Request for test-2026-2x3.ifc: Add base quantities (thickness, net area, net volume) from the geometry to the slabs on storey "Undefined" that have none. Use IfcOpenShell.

First a look at what the model holds.

```python
import ifcopenshell
import ifcopenshell.util.element
import ifcopenshell.util.unit

model = ifcopenshell.open("test-2026-2x3.ifc")
print(model.schema)
for unit_type in ("LENGTHUNIT", "AREAUNIT", "VOLUMEUNIT"):
    print(unit_type, ifcopenshell.util.unit.calculate_unit_scale(model, unit_type))
storey = next(s for s in model.by_type("IfcBuildingStorey") if s.Name == "Undefined")
slabs = [e for e in ifcopenshell.util.element.get_decomposition(storey) if e.is_a("IfcSlab")]
for e in sorted(slabs, key=lambda e: e.id()):
    print(e.id(), e.is_a(), e.Name, list(ifcopenshell.util.element.get_psets(e, qtos_only=True)), sep=" | ")
```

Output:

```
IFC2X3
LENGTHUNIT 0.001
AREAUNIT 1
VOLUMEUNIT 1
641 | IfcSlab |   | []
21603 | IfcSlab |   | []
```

```python
import ifcopenshell
import ifcopenshell.api.pset
import ifcopenshell.geom
import ifcopenshell.util.element
import ifcopenshell.util.shape
import ifcopenshell.util.unit

model = ifcopenshell.open("test-2026-2x3.ifc")
unit_scale = ifcopenshell.util.unit.calculate_unit_scale(model)
area_scale = ifcopenshell.util.unit.calculate_unit_scale(model, "AREAUNIT")
volume_scale = ifcopenshell.util.unit.calculate_unit_scale(model, "VOLUMEUNIT")
settings = ifcopenshell.geom.settings()

storey = next(s for s in model.by_type("IfcBuildingStorey") if s.Name == "Undefined")
slabs = [e for e in ifcopenshell.util.element.get_decomposition(storey) if e.is_a("IfcSlab")]

for e in sorted(slabs, key=lambda e: e.id()):
    if ifcopenshell.util.element.get_psets(e, qtos_only=True, should_inherit=False):
        continue
    # Geometry comes back in metres, in the element's own axes.
    shape = ifcopenshell.geom.create_shape(settings, e)
    values = {
        "Width": ifcopenshell.util.shape.get_z(shape.geometry) / unit_scale,
        "NetArea": ifcopenshell.util.shape.get_footprint_area(shape.geometry) / area_scale,
        "NetVolume": ifcopenshell.util.shape.get_volume(shape.geometry) / volume_scale,
    }
    qto = ifcopenshell.api.pset.add_qto(model, product=e, name="BaseQuantities")
    ifcopenshell.api.pset.edit_qto(model, qto=qto, properties=values)
    print(e.id(), {k: round(v, 3) for k, v in values.items()})

model.write("test-2026-2x3_rev.ifc")
```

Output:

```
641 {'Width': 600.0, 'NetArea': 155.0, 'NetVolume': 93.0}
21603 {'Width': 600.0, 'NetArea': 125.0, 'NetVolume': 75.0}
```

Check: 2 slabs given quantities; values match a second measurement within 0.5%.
